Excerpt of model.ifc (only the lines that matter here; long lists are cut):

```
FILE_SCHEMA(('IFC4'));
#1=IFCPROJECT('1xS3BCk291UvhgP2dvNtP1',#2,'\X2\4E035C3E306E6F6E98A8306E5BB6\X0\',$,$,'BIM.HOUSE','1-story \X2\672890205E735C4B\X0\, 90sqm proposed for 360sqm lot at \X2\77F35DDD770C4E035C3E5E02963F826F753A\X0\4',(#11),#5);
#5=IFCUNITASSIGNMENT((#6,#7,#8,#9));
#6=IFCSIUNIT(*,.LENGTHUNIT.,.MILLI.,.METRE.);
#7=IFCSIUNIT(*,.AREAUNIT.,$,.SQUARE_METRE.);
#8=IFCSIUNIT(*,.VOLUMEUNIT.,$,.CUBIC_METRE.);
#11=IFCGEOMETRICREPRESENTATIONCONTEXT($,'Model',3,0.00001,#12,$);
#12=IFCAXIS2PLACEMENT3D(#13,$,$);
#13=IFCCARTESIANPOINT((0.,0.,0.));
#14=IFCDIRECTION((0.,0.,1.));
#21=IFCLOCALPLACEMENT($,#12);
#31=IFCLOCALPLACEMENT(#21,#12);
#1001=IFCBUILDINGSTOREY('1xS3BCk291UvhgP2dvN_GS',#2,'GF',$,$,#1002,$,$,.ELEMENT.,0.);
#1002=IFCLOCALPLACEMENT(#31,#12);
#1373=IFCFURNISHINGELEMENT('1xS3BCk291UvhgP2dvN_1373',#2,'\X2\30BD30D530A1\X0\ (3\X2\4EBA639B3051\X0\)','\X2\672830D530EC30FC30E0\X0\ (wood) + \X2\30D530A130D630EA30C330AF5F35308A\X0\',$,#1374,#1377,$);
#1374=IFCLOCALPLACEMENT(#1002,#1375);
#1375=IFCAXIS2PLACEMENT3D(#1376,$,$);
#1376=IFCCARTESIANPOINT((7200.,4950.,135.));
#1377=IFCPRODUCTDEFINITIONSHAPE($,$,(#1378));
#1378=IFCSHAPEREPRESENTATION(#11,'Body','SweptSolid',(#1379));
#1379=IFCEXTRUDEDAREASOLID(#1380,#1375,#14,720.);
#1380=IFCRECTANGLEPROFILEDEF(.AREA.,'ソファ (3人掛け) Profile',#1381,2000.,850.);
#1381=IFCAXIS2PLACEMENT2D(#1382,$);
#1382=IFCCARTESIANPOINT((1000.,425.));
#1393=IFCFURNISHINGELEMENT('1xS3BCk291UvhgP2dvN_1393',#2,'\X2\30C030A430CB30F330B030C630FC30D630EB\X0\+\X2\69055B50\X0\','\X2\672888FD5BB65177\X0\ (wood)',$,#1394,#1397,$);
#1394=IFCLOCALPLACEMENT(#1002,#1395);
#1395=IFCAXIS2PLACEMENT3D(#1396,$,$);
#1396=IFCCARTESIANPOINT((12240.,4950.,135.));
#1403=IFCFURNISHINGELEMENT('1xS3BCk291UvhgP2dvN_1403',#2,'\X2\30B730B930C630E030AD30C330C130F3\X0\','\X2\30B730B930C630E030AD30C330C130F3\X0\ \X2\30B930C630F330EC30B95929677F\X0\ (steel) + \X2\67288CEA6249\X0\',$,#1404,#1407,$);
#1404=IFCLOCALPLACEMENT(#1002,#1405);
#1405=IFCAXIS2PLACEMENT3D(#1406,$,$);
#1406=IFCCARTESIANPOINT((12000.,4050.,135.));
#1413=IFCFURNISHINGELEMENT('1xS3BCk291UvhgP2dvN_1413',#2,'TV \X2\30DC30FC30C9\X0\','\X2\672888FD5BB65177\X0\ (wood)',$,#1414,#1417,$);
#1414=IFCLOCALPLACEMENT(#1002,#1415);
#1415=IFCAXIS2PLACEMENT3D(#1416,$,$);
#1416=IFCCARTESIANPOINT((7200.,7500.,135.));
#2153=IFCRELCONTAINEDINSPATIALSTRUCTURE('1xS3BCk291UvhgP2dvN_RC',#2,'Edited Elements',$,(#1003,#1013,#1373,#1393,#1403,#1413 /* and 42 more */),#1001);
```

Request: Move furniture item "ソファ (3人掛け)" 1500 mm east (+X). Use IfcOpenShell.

```python
import ifcopenshell
import ifcopenshell.api.geometry
import ifcopenshell.util.placement

model = ifcopenshell.open("model.ifc")

item = model.by_guid("1xS3BCk291UvhgP2dvN_1373")
matrix = ifcopenshell.util.placement.get_local_placement(item.ObjectPlacement)
matrix[0, 3] += 1500.0
ifcopenshell.api.geometry.edit_object_placement(model, product=item, matrix=matrix, is_si=False)

print(ifcopenshell.util.placement.get_local_placement(item.ObjectPlacement).round(3) + 0.0)

model.write("model_edited.ifc")
```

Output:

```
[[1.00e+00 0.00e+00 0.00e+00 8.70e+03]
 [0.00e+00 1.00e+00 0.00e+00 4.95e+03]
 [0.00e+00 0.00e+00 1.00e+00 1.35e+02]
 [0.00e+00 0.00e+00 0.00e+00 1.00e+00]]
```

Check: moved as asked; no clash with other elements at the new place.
